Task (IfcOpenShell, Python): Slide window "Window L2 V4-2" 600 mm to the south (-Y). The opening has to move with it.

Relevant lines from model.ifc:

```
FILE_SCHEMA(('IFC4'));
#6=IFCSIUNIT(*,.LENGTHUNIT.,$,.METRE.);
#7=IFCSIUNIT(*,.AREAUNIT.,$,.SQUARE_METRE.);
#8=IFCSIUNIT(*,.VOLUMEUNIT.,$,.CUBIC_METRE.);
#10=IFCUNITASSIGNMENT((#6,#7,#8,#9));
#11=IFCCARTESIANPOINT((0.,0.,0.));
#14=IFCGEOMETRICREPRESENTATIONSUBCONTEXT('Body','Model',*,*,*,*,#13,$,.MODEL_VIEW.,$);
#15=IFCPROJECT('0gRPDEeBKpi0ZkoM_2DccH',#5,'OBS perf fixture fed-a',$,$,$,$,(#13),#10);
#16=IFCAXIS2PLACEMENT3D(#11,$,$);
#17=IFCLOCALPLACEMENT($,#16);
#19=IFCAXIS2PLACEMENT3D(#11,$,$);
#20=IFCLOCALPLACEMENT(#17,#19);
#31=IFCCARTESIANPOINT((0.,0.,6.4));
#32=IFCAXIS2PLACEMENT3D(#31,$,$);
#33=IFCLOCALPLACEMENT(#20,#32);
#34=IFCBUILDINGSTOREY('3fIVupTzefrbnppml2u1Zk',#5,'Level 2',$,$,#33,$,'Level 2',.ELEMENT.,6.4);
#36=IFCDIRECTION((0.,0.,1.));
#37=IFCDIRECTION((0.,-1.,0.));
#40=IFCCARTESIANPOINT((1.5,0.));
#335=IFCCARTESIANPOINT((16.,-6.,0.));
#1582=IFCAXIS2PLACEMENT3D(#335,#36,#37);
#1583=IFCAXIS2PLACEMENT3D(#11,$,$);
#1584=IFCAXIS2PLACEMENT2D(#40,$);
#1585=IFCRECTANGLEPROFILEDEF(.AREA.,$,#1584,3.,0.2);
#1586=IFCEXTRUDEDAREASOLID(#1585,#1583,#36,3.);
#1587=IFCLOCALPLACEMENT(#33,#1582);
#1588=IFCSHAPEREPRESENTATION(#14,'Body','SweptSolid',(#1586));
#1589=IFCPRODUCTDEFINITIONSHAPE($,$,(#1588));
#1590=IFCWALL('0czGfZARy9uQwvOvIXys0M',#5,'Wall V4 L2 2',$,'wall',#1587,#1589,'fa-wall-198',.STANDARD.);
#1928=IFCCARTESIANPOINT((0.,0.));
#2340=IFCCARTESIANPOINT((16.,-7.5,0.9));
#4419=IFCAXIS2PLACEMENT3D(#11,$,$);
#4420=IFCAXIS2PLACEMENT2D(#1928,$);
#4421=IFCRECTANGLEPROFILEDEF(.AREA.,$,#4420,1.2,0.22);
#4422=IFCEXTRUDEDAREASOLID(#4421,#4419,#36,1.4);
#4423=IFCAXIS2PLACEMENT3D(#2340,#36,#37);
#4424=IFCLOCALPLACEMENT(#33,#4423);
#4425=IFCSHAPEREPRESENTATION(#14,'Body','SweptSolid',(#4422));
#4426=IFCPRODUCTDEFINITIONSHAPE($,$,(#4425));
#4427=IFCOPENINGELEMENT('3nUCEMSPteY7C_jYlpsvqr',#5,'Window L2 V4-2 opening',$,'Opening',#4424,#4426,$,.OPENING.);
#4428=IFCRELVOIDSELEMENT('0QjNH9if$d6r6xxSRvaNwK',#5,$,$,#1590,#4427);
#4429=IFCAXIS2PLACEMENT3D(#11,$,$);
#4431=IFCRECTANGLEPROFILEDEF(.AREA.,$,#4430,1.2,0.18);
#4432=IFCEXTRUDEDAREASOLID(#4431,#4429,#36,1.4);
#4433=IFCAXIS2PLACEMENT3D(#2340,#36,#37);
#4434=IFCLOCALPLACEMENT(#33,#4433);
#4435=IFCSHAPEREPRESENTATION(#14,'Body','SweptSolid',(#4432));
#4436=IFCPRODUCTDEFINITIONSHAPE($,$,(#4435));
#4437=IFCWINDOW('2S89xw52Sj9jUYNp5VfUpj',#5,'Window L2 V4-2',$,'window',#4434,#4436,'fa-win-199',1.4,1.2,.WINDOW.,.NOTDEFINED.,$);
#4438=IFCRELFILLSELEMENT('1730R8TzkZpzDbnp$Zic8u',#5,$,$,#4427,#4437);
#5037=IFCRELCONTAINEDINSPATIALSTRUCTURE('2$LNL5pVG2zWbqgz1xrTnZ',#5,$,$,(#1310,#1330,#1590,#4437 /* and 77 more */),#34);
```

```python
import ifcopenshell
import ifcopenshell.api.geometry
import ifcopenshell.util.placement

model = ifcopenshell.open("model.ifc")

window = model.by_guid("2S89xw52Sj9jUYNp5VfUpj")
opening = window.FillsVoids[0].RelatingOpeningElement
wall = opening.VoidsElements[0].RelatingBuildingElement

wall_matrix = ifcopenshell.util.placement.get_local_placement(wall.ObjectPlacement)
shift = wall_matrix[:3, 0] * 0.6
before = ifcopenshell.util.placement.get_local_placement(window.ObjectPlacement)[:3, 3].copy()

# The window is not placed relative to its opening, so move both.
for product in (opening, window):
    matrix = ifcopenshell.util.placement.get_local_placement(product.ObjectPlacement)
    matrix[:3, 3] += shift
    ifcopenshell.api.geometry.edit_object_placement(model, product=product, matrix=matrix, is_si=False)

after = ifcopenshell.util.placement.get_local_placement(window.ObjectPlacement)[:3, 3]
print("window moved by", (after - before).round(3) + 0.0)

model.write("model-out.ifc")
```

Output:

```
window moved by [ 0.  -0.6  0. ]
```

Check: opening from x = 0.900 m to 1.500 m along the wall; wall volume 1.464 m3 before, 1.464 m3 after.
